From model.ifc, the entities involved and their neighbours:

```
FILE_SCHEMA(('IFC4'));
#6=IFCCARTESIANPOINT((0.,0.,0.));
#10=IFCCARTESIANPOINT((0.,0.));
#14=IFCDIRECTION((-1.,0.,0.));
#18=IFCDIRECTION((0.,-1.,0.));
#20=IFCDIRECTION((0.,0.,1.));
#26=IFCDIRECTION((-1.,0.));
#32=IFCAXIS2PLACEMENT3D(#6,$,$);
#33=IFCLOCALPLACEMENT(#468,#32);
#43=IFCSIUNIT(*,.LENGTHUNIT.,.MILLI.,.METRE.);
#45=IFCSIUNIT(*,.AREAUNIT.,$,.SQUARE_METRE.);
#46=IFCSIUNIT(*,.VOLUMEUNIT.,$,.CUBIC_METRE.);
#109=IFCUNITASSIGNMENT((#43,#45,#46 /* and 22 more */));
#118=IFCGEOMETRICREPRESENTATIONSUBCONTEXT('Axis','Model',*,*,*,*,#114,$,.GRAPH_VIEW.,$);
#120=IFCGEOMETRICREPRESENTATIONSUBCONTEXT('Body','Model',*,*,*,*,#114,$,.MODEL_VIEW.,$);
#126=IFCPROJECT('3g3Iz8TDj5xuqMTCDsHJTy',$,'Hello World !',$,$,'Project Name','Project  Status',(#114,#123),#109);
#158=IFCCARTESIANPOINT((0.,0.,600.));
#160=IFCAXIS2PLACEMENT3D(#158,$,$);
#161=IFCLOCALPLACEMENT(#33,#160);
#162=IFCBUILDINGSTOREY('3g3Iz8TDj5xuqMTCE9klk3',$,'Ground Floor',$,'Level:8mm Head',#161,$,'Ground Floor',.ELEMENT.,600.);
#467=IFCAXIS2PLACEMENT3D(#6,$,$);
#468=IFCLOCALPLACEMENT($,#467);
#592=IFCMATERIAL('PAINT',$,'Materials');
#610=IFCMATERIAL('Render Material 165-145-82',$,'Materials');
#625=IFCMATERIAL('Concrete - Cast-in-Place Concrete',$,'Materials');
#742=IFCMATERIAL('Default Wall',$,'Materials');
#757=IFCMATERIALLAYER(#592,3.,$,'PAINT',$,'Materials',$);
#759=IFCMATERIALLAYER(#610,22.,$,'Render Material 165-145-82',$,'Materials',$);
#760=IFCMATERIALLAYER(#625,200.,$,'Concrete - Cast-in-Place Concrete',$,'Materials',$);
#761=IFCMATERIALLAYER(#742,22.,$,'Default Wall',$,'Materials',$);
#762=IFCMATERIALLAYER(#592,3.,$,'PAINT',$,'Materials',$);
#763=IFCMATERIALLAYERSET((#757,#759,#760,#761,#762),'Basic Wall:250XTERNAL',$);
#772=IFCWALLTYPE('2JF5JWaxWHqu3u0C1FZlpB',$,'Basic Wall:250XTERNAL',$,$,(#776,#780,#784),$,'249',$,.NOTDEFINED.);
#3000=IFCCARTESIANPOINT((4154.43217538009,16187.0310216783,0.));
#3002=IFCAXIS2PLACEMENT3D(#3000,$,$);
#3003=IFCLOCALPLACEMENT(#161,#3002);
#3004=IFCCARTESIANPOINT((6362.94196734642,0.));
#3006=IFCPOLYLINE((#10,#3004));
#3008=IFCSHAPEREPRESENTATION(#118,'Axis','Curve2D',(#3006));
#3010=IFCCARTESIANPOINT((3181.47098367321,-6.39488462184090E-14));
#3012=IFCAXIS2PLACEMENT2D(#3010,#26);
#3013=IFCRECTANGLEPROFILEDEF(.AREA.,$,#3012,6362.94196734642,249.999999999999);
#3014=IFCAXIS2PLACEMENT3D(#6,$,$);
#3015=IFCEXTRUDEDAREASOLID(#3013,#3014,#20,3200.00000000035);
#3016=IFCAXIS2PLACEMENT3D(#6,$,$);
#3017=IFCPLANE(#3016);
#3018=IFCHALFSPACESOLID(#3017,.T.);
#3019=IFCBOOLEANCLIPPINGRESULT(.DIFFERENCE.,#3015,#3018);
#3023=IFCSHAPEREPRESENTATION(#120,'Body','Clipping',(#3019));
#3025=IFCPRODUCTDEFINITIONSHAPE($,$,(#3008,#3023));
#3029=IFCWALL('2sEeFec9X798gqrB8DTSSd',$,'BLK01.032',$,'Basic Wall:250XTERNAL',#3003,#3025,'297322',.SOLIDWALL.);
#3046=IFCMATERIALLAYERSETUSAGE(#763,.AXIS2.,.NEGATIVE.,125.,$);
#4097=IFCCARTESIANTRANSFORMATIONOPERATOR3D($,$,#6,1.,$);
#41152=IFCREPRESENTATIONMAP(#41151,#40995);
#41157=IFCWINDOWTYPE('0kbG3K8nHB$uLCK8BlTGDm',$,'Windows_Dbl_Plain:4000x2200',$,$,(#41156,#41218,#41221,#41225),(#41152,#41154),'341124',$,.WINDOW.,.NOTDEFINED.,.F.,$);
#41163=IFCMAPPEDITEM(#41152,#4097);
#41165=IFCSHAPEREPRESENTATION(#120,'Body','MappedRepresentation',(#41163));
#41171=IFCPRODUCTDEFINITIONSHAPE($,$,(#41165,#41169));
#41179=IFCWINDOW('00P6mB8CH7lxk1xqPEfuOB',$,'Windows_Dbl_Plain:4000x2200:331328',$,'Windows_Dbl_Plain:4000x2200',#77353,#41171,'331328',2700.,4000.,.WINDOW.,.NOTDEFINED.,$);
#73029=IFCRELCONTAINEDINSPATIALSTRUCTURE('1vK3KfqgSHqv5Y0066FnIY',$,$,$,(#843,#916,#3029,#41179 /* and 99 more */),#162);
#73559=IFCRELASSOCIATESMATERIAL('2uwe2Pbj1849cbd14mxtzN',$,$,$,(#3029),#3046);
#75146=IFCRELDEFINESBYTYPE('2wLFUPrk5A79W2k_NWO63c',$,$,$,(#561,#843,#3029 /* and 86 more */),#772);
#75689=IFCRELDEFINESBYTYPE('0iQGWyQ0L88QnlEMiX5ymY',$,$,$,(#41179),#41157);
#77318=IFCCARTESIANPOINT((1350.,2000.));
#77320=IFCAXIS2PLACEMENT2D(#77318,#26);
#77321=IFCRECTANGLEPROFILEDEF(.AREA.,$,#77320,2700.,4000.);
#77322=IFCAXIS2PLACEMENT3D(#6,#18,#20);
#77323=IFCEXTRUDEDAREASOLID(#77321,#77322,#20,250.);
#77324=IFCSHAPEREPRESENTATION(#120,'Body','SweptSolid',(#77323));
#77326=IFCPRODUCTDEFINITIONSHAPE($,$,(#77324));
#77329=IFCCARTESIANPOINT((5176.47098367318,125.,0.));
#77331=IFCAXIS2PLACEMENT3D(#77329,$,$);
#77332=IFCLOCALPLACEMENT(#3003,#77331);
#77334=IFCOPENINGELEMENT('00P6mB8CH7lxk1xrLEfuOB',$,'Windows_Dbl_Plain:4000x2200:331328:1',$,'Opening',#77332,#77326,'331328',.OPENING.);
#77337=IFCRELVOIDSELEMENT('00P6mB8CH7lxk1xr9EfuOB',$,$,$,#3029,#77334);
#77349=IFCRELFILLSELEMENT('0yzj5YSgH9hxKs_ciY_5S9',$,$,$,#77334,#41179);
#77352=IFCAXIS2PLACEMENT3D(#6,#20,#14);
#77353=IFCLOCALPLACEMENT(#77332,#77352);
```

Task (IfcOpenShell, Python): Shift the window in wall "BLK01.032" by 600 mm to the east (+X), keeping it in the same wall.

```python
import ifcopenshell
import ifcopenshell.api.geometry
import ifcopenshell.util.placement
import ifcopenshell.util.unit

model = ifcopenshell.open("model.ifc")
unit_scale = ifcopenshell.util.unit.calculate_unit_scale(model)

window = model.by_guid("00P6mB8CH7lxk1xqPEfuOB")
opening = window.FillsVoids[0].RelatingOpeningElement
wall = opening.VoidsElements[0].RelatingBuildingElement

wall_matrix = ifcopenshell.util.placement.get_local_placement(wall.ObjectPlacement)
shift = wall_matrix[:3, 0] * 0.6 / unit_scale
before = ifcopenshell.util.placement.get_local_placement(window.ObjectPlacement)[:3, 3].copy()

# The window is placed relative to its opening, so it follows when the opening moves.
matrix = ifcopenshell.util.placement.get_local_placement(opening.ObjectPlacement)
matrix[:3, 3] += shift
ifcopenshell.api.geometry.edit_object_placement(
    model, product=opening, matrix=matrix, is_si=False, should_transform_children=True
)

after = ifcopenshell.util.placement.get_local_placement(window.ObjectPlacement)[:3, 3]
print("window moved by", (after - before).round(3) + 0.0)

model.write("model_v2.ifc")
```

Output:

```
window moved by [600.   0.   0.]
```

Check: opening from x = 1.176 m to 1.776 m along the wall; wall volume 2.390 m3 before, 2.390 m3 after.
